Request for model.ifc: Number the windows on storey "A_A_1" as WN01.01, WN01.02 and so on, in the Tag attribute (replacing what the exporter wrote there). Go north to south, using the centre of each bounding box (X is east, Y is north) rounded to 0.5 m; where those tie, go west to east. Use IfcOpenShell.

First a look at what the model holds.

```python
import ifcopenshell
import ifcopenshell.util.element
import ifcopenshell.util.placement

model = ifcopenshell.open("model.ifc")
print(model.schema)
storey = next(s for s in model.by_type("IfcBuildingStorey") if s.Name == "A_A_1")
windows = [e for e in ifcopenshell.util.element.get_decomposition(storey) if e.is_a("IfcWindow")]
for e in sorted(windows, key=lambda e: e.id()):
    origin = ifcopenshell.util.placement.get_local_placement(e.ObjectPlacement)[:3, 3]
    print(e.id(), e.Tag, e.Name, origin.round(2) + 0.0, sep=" | ")
```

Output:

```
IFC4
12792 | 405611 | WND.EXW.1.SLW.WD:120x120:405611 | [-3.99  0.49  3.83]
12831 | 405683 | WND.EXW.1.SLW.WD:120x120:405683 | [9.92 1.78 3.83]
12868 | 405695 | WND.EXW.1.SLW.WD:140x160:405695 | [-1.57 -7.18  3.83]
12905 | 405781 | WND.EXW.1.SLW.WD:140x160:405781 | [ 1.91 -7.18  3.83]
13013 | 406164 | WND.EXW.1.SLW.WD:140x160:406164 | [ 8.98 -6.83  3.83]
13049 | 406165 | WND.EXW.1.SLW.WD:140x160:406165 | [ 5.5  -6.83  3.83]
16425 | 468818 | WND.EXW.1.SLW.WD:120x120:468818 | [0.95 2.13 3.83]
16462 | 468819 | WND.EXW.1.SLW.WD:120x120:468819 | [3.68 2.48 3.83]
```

```python
import ifcopenshell
import ifcopenshell.geom
import ifcopenshell.util.element
import ifcopenshell.util.shape

model = ifcopenshell.open("model.ifc")
settings = ifcopenshell.geom.settings()
settings.set("use-world-coords", True)


def centre(element):
    shape = ifcopenshell.geom.create_shape(settings, element)
    return ifcopenshell.util.shape.get_bbox_centroid(shape.geometry)


storey = next(s for s in model.by_type("IfcBuildingStorey") if s.Name == "A_A_1")
windows = [e for e in ifcopenshell.util.element.get_decomposition(storey) if e.is_a("IfcWindow")]

# Insertion points can sit at a corner or the storey origin, so sort by the geometry (in metres).
centres = {e: centre(e) for e in windows}
windows.sort(key=lambda e: (-round(centres[e][1] / 0.5), centres[e][0]))

for i, e in enumerate(windows, start=1):
    number = f"WN01.{i:02d}"
    e.Tag = number
    print(e.id(), number)

model.write("model_updated.ifc")
```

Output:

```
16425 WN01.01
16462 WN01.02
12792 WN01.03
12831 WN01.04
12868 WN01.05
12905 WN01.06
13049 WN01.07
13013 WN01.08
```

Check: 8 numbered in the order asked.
